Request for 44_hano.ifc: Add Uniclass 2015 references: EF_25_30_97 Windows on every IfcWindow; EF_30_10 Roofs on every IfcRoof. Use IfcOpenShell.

First a look at what the model holds.

```python
import ifcopenshell

model = ifcopenshell.open("44_hano.ifc")
print(model.schema)
print("classifications:", [c.Name for c in model.by_type("IfcClassification")])
for ifc_class in ("IfcDoor", "IfcRoof", "IfcStair", "IfcWall", "IfcWindow"):
    print(ifc_class, len(model.by_type(ifc_class)))
```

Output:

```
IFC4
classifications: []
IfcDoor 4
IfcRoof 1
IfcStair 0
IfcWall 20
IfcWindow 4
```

```python
import ifcopenshell
import ifcopenshell.api.classification

model = ifcopenshell.open("44_hano.ifc")

system = ifcopenshell.api.classification.add_classification(model, classification="Uniclass 2015")

codes = {
    "IfcWindow": ("EF_25_30_97", "Windows"),
    "IfcRoof": ("EF_30_10", "Roofs"),
}
for ifc_class, (code, name) in codes.items():
    products = model.by_type(ifc_class)
    ifcopenshell.api.classification.add_reference(
        model, products=products, classification=system, identification=code, name=name
    )
    print(code, len(products))

model.write("44_hano_edited.ifc")
```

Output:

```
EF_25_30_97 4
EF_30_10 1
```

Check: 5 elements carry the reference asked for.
